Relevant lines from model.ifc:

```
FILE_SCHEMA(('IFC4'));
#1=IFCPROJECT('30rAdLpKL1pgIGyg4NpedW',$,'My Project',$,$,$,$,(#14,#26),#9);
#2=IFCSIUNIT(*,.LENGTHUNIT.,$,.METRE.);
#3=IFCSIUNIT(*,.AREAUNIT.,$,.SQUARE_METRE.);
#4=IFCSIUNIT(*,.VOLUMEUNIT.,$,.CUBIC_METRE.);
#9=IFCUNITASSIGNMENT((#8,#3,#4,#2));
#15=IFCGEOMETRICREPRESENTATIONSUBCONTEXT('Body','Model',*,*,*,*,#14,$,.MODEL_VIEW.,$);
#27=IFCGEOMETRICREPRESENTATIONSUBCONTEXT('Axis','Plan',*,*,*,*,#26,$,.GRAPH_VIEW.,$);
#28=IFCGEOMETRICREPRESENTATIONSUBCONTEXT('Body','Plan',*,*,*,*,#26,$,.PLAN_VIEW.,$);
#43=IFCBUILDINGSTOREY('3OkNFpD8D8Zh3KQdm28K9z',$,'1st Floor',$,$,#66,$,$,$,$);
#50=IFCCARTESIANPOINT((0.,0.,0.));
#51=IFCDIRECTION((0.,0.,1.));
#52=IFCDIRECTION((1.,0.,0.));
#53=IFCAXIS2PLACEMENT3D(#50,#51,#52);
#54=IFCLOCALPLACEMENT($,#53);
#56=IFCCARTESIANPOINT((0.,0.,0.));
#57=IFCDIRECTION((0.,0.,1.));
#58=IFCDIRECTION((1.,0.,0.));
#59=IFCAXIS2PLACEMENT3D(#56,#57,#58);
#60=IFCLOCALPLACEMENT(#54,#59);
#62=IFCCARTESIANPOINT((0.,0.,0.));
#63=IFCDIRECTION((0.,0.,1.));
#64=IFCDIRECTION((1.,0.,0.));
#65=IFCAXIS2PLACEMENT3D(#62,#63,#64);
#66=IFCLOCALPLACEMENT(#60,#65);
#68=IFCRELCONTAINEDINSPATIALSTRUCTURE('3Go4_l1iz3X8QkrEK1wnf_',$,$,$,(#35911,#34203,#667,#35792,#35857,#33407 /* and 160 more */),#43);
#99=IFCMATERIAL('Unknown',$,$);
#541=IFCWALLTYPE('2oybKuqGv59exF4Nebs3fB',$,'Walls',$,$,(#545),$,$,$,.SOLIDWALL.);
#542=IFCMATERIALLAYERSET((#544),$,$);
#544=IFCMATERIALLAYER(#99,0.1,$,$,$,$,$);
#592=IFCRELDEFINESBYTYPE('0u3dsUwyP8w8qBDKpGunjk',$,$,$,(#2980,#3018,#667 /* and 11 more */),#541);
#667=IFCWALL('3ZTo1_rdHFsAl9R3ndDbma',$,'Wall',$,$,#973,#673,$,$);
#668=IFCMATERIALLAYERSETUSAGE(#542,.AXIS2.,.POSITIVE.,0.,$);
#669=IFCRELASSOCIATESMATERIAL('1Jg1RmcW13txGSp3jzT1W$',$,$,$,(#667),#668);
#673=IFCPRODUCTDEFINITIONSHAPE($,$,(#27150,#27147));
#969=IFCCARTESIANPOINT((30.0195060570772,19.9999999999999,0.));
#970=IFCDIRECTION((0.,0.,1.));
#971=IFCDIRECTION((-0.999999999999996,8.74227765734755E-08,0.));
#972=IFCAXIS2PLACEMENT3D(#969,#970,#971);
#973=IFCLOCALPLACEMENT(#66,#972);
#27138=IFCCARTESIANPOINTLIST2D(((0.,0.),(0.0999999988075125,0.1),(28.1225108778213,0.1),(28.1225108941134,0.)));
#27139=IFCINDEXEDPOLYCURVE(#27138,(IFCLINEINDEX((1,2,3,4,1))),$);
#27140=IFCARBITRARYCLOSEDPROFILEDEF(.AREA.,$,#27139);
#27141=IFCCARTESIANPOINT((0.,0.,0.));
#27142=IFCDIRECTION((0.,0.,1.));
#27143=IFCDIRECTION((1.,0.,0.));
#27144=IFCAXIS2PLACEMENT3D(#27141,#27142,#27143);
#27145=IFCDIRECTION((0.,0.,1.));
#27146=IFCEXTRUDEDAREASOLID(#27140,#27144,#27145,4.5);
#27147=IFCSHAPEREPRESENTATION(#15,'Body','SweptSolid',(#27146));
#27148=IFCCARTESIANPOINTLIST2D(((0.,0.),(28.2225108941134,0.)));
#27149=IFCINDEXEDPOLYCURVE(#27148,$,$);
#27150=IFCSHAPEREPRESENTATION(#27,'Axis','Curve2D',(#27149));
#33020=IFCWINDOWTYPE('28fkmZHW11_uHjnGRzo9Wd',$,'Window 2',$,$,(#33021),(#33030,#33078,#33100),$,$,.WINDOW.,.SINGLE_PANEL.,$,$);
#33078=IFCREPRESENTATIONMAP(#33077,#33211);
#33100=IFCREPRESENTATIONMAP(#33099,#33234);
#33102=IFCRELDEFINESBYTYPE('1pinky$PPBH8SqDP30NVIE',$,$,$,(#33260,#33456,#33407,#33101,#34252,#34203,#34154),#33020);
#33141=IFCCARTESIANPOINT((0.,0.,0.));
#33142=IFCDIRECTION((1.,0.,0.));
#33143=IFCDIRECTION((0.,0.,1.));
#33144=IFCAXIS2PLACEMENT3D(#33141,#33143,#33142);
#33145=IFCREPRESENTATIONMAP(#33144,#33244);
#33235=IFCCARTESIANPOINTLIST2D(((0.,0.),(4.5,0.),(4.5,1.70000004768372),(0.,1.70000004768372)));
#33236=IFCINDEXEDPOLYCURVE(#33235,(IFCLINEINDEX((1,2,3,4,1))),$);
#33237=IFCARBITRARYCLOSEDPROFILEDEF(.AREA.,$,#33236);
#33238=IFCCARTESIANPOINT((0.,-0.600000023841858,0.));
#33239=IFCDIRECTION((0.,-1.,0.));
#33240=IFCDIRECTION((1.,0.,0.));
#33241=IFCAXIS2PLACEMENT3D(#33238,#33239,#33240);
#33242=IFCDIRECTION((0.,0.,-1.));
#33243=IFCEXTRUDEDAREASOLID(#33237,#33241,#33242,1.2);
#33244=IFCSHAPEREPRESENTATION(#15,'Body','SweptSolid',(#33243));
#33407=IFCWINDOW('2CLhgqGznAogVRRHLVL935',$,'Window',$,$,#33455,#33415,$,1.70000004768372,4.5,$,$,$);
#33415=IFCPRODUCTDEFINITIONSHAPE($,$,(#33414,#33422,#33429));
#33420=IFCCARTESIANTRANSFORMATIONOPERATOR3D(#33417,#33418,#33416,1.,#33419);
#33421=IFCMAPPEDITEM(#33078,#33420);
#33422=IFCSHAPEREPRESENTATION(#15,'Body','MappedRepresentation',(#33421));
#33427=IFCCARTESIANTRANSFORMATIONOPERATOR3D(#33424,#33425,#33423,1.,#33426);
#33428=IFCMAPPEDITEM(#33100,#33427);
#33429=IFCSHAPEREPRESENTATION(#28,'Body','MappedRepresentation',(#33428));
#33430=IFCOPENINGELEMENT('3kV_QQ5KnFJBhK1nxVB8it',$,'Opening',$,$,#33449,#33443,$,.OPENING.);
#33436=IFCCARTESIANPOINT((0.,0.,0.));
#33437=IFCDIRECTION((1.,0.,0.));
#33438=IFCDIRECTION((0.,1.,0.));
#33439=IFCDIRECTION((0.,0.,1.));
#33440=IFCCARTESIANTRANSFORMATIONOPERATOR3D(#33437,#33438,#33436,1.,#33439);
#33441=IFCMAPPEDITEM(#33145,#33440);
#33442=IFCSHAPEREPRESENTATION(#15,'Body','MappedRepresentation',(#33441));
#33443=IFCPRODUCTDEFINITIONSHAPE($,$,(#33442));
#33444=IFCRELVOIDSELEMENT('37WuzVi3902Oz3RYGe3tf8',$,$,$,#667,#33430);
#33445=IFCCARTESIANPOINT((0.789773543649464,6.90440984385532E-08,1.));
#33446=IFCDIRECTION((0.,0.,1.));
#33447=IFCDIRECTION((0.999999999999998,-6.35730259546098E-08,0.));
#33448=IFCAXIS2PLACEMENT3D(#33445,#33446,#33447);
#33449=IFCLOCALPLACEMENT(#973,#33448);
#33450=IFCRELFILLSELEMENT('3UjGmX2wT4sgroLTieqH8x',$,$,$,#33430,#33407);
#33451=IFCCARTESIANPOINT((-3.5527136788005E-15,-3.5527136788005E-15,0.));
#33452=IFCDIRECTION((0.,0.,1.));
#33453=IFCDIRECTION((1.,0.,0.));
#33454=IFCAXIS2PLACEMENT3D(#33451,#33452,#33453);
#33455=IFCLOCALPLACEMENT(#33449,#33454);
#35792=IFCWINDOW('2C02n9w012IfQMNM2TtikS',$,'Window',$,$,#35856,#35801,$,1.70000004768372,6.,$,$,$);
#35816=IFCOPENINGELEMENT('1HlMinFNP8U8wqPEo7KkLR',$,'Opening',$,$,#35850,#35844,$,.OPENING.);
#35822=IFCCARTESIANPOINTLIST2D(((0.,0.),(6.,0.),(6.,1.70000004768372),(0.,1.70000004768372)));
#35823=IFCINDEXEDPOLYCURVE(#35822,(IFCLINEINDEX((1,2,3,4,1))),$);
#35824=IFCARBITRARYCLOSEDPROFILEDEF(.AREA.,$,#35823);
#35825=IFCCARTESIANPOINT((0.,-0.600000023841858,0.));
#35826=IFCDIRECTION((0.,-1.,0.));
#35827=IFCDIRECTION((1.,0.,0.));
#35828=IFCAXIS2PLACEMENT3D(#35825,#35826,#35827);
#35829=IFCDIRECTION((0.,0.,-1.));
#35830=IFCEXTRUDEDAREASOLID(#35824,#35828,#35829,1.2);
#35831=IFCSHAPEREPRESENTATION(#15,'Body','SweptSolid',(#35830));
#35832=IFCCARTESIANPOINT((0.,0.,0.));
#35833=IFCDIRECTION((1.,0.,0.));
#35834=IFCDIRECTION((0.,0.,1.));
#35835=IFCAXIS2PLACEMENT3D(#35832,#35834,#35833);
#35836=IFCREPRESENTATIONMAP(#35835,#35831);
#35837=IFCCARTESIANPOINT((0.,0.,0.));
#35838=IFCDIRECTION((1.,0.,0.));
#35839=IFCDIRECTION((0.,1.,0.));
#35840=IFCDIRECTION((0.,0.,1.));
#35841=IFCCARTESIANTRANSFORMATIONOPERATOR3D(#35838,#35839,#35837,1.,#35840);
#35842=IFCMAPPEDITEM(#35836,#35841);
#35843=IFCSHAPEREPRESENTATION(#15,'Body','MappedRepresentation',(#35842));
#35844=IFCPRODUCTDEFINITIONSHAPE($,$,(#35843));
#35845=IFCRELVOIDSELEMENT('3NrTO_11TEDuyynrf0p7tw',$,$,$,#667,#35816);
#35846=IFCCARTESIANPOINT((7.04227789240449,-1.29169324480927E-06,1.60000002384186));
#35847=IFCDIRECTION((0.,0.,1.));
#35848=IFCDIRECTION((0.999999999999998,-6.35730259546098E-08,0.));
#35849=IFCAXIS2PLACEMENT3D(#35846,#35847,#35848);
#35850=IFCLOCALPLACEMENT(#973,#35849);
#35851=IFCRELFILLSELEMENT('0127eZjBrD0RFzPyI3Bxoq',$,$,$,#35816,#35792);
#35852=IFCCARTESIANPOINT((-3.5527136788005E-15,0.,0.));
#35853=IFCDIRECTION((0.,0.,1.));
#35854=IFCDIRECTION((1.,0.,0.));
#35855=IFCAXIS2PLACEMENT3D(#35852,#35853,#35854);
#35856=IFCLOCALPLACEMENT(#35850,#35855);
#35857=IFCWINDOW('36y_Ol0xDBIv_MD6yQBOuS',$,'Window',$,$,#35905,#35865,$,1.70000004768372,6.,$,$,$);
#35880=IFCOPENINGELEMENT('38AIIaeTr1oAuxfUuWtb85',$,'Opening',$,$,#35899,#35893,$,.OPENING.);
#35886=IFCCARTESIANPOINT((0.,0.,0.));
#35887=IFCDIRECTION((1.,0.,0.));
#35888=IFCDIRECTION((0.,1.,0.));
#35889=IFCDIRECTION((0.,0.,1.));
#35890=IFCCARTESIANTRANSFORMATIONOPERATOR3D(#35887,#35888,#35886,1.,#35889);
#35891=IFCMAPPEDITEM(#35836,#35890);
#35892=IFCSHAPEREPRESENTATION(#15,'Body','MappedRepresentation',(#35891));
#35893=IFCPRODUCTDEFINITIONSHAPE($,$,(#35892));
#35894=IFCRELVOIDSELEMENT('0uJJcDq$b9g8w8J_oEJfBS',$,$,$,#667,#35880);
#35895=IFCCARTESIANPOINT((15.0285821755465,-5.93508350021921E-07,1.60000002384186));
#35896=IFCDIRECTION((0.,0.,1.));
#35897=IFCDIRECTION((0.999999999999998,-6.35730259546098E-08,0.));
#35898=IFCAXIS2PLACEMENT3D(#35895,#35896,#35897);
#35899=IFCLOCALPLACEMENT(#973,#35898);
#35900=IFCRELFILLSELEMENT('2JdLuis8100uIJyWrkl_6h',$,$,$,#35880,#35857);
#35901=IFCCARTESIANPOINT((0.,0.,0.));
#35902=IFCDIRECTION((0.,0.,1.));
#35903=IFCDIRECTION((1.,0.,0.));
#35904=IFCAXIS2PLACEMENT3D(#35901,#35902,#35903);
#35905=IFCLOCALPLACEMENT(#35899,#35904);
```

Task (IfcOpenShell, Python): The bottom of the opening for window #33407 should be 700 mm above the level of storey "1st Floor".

```python
import numpy as np
import ifcopenshell
import ifcopenshell.api.geometry
import ifcopenshell.geom
import ifcopenshell.util.element
import ifcopenshell.util.placement
import ifcopenshell.util.shape
import ifcopenshell.util.unit

model = ifcopenshell.open("model.ifc")
unit_scale = ifcopenshell.util.unit.calculate_unit_scale(model)

window = model.by_guid("2CLhgqGznAogVRRHLVL935")
opening = window.FillsVoids[0].RelatingOpeningElement
storey = ifcopenshell.util.element.get_container(window, ifc_class="IfcBuildingStorey")
level = ifcopenshell.util.placement.get_local_placement(storey.ObjectPlacement)[2, 3]

# The opening's origin need not be at the sill, so measure its lowest point.
shape = ifcopenshell.geom.create_shape(ifcopenshell.geom.settings(), opening)
bottom = ifcopenshell.util.shape.get_shape_bottom_elevation(shape, shape.geometry) / unit_scale
dz = level + 0.7 - bottom

shift = np.array([0.0, 0.0, dz])
# The window is placed relative to its opening, so it follows when the opening moves.
matrix = ifcopenshell.util.placement.get_local_placement(opening.ObjectPlacement)
matrix[:3, 3] += shift
ifcopenshell.api.geometry.edit_object_placement(
    model, product=opening, matrix=matrix, is_si=False, should_transform_children=True
)

print(f"moved by {dz * unit_scale:+.3f} m")

model.write("model_v2.ifc")
```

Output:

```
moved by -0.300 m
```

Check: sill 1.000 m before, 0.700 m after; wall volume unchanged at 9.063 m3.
